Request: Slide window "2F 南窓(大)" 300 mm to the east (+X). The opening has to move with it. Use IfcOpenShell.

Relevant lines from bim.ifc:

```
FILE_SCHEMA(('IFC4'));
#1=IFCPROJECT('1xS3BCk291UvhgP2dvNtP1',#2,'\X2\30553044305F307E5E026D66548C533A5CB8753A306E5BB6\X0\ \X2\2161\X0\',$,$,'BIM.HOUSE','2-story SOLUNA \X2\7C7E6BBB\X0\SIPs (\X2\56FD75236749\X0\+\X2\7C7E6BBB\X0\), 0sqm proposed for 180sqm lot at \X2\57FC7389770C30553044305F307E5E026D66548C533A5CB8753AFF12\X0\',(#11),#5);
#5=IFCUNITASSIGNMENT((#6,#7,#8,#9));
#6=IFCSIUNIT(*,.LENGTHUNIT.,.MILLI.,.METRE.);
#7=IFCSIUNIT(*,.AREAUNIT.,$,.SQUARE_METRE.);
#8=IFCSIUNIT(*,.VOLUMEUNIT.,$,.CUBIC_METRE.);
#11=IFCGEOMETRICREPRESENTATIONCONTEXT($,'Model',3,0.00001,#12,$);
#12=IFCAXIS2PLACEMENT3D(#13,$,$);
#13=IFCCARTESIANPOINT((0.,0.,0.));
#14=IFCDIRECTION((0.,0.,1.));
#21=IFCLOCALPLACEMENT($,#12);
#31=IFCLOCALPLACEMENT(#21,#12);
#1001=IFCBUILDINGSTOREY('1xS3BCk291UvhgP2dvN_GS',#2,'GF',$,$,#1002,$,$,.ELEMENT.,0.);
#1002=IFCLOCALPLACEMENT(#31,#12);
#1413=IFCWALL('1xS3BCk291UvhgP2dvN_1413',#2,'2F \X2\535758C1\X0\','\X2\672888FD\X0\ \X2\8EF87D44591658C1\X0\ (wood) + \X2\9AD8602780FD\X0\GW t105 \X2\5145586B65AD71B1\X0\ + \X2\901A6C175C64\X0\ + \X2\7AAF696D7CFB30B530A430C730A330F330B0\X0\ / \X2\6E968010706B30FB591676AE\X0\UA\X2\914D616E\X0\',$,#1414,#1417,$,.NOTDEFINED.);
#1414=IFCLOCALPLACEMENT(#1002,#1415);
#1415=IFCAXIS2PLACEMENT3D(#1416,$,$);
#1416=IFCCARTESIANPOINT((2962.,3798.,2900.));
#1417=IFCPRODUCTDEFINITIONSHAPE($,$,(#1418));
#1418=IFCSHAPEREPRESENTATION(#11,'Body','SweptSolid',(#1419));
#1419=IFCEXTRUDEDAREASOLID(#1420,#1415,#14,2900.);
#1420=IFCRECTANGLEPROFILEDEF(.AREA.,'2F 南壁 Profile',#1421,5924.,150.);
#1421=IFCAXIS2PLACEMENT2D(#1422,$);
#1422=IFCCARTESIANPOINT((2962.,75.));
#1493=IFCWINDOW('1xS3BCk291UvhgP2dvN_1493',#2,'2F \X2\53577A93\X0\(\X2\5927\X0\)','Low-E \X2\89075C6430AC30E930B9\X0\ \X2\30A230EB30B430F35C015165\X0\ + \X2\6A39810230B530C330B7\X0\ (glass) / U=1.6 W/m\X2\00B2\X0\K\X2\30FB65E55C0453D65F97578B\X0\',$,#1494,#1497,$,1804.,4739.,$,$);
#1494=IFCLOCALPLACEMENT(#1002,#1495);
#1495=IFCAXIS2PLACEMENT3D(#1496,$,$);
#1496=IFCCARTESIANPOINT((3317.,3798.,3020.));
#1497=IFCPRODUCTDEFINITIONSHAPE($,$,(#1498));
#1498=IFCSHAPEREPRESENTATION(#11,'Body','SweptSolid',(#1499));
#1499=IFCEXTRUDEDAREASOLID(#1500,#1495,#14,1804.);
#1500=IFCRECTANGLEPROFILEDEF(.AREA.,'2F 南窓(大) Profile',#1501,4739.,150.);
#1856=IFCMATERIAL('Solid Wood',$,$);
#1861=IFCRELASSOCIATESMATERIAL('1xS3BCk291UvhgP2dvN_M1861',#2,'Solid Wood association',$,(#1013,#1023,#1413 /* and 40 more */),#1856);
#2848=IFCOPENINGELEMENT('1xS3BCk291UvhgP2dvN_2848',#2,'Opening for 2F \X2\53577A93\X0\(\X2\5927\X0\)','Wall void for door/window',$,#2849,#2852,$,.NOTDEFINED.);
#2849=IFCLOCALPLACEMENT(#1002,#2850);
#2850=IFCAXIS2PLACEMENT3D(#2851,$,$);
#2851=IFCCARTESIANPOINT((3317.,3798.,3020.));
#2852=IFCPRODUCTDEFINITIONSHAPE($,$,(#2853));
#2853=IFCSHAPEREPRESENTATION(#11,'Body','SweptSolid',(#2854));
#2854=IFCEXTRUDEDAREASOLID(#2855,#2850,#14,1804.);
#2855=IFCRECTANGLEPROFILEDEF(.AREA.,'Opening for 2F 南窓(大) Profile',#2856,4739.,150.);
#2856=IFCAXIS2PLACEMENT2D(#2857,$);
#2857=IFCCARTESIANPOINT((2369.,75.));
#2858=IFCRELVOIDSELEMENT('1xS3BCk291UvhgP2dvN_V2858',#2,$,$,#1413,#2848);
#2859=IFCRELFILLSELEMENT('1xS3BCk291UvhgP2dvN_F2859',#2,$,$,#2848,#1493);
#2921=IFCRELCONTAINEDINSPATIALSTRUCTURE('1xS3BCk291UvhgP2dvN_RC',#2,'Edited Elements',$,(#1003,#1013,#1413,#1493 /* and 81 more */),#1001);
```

```python
import ifcopenshell
import ifcopenshell.api.geometry
import ifcopenshell.util.placement

model = ifcopenshell.open("bim.ifc")

window = model.by_guid("1xS3BCk291UvhgP2dvN_1493")
opening = window.FillsVoids[0].RelatingOpeningElement
wall = opening.VoidsElements[0].RelatingBuildingElement

wall_matrix = ifcopenshell.util.placement.get_local_placement(wall.ObjectPlacement)
shift = wall_matrix[:3, 0] * 300.0
before = ifcopenshell.util.placement.get_local_placement(window.ObjectPlacement)[:3, 3].copy()

# The window is not placed relative to its opening, so move both.
for product in (opening, window):
    matrix = ifcopenshell.util.placement.get_local_placement(product.ObjectPlacement)
    matrix[:3, 3] += shift
    ifcopenshell.api.geometry.edit_object_placement(model, product=product, matrix=matrix, is_si=False)

after = ifcopenshell.util.placement.get_local_placement(window.ObjectPlacement)[:3, 3]
print("window moved by", (after - before).round(3) + 0.0)

model.write("bim-out.ifc")
```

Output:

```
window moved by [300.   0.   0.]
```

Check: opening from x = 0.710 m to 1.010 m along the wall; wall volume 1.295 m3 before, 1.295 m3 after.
